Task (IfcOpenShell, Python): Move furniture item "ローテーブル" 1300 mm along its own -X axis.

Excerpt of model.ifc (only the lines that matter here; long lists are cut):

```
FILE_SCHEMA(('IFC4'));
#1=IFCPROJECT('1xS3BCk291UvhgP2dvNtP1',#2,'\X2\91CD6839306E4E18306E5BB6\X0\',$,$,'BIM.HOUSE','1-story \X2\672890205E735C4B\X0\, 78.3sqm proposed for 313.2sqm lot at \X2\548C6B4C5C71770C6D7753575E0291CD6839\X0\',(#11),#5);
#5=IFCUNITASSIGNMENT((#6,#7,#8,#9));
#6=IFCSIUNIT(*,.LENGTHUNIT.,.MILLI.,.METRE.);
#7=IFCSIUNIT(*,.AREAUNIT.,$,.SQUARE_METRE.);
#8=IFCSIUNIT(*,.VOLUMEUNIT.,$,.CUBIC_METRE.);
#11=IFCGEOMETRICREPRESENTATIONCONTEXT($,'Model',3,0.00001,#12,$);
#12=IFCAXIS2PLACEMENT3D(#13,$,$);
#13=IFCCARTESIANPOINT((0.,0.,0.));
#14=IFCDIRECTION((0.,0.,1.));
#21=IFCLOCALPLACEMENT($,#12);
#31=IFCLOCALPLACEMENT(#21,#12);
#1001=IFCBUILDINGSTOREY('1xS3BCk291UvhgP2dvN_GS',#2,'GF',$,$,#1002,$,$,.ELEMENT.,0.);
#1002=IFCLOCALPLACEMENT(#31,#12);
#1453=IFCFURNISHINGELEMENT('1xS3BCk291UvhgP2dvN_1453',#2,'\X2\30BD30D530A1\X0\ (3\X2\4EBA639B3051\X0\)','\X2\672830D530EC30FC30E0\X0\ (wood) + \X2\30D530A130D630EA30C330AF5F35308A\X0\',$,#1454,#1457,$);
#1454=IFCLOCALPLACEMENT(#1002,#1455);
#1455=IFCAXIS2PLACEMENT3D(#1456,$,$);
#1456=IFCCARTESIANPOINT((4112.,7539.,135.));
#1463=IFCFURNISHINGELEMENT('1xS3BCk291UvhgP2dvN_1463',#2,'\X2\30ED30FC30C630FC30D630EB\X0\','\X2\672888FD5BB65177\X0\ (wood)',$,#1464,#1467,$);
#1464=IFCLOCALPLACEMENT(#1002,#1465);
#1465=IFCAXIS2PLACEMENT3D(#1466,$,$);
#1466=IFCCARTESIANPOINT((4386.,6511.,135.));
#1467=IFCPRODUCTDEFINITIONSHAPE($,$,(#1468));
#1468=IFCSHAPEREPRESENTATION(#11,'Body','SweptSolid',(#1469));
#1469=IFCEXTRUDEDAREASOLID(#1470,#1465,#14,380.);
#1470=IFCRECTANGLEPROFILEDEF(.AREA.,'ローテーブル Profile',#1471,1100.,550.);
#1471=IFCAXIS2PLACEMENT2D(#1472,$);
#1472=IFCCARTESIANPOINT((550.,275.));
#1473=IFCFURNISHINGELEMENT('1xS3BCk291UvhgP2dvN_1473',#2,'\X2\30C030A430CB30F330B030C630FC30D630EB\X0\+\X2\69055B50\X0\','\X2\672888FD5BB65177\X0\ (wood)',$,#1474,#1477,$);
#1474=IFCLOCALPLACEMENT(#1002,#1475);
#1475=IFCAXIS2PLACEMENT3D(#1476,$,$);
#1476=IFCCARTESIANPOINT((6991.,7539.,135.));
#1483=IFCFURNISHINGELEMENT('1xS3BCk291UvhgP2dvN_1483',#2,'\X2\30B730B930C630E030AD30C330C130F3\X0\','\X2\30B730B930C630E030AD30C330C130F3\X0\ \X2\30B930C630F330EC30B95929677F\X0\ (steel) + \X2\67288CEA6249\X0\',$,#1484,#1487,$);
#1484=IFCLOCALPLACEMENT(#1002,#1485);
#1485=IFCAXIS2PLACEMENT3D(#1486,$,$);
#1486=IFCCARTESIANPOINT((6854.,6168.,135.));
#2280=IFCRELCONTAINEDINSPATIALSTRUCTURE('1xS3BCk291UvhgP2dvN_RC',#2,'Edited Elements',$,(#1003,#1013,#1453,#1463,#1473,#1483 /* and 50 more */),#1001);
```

```python
import ifcopenshell
import ifcopenshell.api.geometry
import ifcopenshell.util.placement

model = ifcopenshell.open("model.ifc")

item = model.by_guid("1xS3BCk291UvhgP2dvN_1463")
matrix = ifcopenshell.util.placement.get_local_placement(item.ObjectPlacement)
matrix[:3, 3] -= matrix[:3, 0] * 1300.0
ifcopenshell.api.geometry.edit_object_placement(model, product=item, matrix=matrix, is_si=False)

print(ifcopenshell.util.placement.get_local_placement(item.ObjectPlacement).round(3) + 0.0)

model.write("model_v2.ifc")
```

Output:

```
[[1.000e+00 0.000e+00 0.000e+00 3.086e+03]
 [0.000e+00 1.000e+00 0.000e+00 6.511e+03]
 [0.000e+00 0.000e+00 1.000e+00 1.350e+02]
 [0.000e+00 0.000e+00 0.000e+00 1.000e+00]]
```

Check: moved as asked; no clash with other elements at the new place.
